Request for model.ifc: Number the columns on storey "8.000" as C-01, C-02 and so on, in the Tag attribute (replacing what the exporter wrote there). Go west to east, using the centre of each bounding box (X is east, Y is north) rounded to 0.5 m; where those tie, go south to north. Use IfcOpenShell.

First a look at what the model holds.

```python
import ifcopenshell
import ifcopenshell.util.element
import ifcopenshell.util.placement

model = ifcopenshell.open("model.ifc")
print(model.schema)
storey = next(s for s in model.by_type("IfcBuildingStorey") if s.Name == "8.000")
columns = [e for e in ifcopenshell.util.element.get_decomposition(storey) if e.is_a("IfcColumn")]
for e in sorted(columns, key=lambda e: e.id()):
    origin = ifcopenshell.util.placement.get_local_placement(e.ObjectPlacement)[:3, 3]
    print(e.id(), e.Tag, e.Name, origin.round(2) + 0.0, sep=" | ")
```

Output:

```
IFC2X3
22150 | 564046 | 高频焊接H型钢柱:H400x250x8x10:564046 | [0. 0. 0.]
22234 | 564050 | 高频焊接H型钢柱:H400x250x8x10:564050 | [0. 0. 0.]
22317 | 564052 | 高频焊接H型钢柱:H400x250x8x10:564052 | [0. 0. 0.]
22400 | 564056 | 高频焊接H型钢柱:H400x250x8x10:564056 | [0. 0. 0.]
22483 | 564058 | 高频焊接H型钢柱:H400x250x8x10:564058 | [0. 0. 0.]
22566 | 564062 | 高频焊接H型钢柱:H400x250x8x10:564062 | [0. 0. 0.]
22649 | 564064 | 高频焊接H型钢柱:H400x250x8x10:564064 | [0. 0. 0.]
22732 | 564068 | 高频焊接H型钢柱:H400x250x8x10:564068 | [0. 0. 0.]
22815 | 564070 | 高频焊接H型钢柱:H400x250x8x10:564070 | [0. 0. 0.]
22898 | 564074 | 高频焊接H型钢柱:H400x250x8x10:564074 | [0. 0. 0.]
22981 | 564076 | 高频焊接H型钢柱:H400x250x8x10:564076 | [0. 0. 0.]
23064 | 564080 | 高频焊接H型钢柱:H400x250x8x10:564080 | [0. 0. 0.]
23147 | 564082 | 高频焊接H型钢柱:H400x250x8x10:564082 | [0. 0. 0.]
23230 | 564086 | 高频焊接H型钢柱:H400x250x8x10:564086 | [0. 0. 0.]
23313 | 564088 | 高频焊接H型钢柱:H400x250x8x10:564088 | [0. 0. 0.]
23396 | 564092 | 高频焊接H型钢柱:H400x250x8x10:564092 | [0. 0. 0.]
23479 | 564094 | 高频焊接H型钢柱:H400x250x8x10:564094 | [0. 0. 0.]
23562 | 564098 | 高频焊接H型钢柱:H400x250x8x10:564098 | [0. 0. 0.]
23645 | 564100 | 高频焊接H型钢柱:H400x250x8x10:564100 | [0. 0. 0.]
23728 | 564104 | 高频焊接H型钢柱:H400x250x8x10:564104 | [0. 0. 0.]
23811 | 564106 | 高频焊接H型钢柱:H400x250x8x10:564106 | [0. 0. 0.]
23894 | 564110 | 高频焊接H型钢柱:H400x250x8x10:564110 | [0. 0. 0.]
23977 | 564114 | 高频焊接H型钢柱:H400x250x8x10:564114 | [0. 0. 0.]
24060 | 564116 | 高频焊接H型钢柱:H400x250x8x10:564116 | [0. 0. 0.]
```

```python
import ifcopenshell
import ifcopenshell.geom
import ifcopenshell.util.element
import ifcopenshell.util.shape

model = ifcopenshell.open("model.ifc")
settings = ifcopenshell.geom.settings()
settings.set("use-world-coords", True)


def centre(element):
    shape = ifcopenshell.geom.create_shape(settings, element)
    return ifcopenshell.util.shape.get_bbox_centroid(shape.geometry)


storey = next(s for s in model.by_type("IfcBuildingStorey") if s.Name == "8.000")
columns = [e for e in ifcopenshell.util.element.get_decomposition(storey) if e.is_a("IfcColumn")]

# Insertion points can sit at a corner or the storey origin, so sort by the geometry (in metres).
centres = {e: centre(e) for e in columns}
columns.sort(key=lambda e: (round(centres[e][0] / 0.5), centres[e][1]))

for i, e in enumerate(columns, start=1):
    number = f"C-{i:02d}"
    e.Tag = number
    print(e.id(), number)

model.write("model_rev.ifc")
```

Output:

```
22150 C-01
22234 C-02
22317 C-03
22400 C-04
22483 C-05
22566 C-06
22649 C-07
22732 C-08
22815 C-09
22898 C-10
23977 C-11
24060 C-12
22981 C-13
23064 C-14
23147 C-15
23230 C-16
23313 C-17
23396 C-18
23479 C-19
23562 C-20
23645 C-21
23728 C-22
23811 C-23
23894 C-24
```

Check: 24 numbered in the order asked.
